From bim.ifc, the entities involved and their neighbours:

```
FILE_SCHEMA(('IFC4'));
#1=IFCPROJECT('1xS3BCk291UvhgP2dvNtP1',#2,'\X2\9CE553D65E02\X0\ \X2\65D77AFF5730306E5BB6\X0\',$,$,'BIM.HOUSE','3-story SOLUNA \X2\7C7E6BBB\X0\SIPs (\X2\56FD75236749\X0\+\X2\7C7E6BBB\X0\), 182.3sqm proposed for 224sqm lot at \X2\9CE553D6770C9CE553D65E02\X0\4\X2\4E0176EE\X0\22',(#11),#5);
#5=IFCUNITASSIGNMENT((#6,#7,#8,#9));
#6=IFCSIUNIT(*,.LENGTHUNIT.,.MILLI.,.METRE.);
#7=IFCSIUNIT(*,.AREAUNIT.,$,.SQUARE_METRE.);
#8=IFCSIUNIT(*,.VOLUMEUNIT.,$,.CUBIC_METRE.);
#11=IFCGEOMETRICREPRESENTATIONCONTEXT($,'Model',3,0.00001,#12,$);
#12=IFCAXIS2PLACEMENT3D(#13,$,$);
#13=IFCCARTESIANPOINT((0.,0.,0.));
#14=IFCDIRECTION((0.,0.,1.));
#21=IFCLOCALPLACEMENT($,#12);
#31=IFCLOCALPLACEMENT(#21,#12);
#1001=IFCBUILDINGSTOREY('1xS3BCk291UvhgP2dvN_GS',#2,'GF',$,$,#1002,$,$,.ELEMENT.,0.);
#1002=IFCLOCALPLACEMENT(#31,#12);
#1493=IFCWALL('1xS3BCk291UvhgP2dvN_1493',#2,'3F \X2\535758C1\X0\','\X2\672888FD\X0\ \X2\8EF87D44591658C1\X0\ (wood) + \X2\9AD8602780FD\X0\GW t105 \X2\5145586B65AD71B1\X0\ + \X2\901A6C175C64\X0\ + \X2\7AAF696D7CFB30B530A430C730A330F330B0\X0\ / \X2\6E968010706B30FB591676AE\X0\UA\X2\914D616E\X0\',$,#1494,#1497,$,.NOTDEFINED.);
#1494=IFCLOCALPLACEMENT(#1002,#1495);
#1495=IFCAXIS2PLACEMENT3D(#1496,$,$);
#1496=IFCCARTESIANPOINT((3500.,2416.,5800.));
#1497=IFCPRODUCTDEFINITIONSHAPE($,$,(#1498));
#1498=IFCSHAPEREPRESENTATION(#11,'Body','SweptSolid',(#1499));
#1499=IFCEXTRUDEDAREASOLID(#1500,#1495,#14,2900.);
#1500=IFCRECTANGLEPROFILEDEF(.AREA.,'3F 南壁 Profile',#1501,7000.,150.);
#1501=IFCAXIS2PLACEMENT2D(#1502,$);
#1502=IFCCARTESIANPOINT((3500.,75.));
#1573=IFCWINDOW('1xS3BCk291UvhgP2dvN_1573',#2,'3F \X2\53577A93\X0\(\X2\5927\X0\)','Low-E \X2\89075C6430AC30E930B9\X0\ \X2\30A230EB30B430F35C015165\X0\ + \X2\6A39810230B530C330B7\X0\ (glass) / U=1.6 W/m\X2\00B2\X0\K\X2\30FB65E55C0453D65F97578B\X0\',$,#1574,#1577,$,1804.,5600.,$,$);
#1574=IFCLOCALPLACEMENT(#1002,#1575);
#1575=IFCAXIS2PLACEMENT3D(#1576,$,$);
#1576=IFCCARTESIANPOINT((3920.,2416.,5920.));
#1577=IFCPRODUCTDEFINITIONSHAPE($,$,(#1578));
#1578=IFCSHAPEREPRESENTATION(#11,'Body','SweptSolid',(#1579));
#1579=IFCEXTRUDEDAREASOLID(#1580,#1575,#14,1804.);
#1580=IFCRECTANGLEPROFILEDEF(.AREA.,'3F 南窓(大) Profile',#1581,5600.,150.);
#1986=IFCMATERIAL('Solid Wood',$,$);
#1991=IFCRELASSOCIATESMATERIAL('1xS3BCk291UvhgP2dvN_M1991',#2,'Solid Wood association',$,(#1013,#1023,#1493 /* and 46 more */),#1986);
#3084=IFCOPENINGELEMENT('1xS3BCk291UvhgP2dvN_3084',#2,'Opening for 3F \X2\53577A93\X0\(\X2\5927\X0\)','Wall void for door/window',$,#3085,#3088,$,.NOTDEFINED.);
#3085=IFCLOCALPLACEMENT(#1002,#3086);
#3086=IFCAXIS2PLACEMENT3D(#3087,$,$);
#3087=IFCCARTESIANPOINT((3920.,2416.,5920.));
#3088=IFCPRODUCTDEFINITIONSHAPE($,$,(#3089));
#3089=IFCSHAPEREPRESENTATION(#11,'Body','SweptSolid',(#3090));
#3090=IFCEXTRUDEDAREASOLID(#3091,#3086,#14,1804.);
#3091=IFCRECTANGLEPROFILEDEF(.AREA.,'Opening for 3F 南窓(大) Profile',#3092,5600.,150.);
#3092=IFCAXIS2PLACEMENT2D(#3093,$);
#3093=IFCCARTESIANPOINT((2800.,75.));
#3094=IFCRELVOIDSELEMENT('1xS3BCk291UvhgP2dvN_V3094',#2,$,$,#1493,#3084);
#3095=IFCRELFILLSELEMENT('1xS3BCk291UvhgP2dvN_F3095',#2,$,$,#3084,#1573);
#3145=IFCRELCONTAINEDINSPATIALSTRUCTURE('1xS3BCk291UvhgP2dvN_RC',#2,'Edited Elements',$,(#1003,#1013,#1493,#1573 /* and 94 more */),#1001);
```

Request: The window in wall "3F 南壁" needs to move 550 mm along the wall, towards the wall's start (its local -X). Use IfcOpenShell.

```python
import ifcopenshell
import ifcopenshell.api.geometry
import ifcopenshell.util.placement
import ifcopenshell.util.unit

model = ifcopenshell.open("bim.ifc")
unit_scale = ifcopenshell.util.unit.calculate_unit_scale(model)

window = model.by_guid("1xS3BCk291UvhgP2dvN_1573")
opening = window.FillsVoids[0].RelatingOpeningElement
wall = opening.VoidsElements[0].RelatingBuildingElement

wall_matrix = ifcopenshell.util.placement.get_local_placement(wall.ObjectPlacement)
shift = wall_matrix[:3, 0] * -0.55 / unit_scale
before = ifcopenshell.util.placement.get_local_placement(window.ObjectPlacement)[:3, 3].copy()

# The window is not placed relative to its opening, so move both.
for product in (opening, window):
    matrix = ifcopenshell.util.placement.get_local_placement(product.ObjectPlacement)
    matrix[:3, 3] += shift
    ifcopenshell.api.geometry.edit_object_placement(model, product=product, matrix=matrix, is_si=False)

after = ifcopenshell.util.placement.get_local_placement(window.ObjectPlacement)[:3, 3]
print("window moved by", (after - before).round(3) + 0.0)

model.write("bim_rev.ifc")
```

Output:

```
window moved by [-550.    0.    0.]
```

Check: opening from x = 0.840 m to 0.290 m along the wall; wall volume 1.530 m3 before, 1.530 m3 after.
